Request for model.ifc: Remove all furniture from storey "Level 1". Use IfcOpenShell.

First a look at what the model holds.

```python
import ifcopenshell
import ifcopenshell.util.element

model = ifcopenshell.open("model.ifc")
print(model.schema)
storey = next(s for s in model.by_type("IfcBuildingStorey") if s.Name == "Level 1")
furniture = [e for e in ifcopenshell.util.element.get_decomposition(storey) if e.is_a("IfcFurnishingElement")]
seen = {}
for e in furniture:
    element_type = ifcopenshell.util.element.get_type(e)
    name = element_type.Name if element_type not in (None, e) else None
    seen[name] = seen.get(name, 0) + 1
for name, count in sorted(seen.items(), key=str):
    print(count, "x", name)
```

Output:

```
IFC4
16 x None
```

```python
import ifcopenshell
import ifcopenshell.api.root
import ifcopenshell.util.element

model = ifcopenshell.open("model.ifc")

storey = next(s for s in model.by_type("IfcBuildingStorey") if s.Name == "Level 1")
furniture = [e for e in ifcopenshell.util.element.get_decomposition(storey) if e.is_a("IfcFurnishingElement")]

for e in furniture:
    ifcopenshell.api.root.remove_product(model, product=e)
print(len(furniture), "removed")

model.write("model_v2.ifc")
```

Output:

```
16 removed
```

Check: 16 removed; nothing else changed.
